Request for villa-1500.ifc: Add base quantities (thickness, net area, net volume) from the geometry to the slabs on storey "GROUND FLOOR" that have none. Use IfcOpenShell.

First a look at what the model holds.

```python
import ifcopenshell
import ifcopenshell.util.element
import ifcopenshell.util.unit

model = ifcopenshell.open("villa-1500.ifc")
print(model.schema)
for unit_type in ("LENGTHUNIT", "AREAUNIT", "VOLUMEUNIT"):
    print(unit_type, ifcopenshell.util.unit.calculate_unit_scale(model, unit_type))
storey = next(s for s in model.by_type("IfcBuildingStorey") if s.Name == "GROUND FLOOR")
slabs = [e for e in ifcopenshell.util.element.get_decomposition(storey) if e.is_a("IfcSlab")]
for e in sorted(slabs, key=lambda e: e.id()):
    print(e.id(), e.is_a(), e.Name, list(ifcopenshell.util.element.get_psets(e, qtos_only=True)), sep=" | ")
```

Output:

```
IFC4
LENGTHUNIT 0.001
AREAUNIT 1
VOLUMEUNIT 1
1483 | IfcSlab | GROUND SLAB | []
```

```python
import ifcopenshell
import ifcopenshell.api.pset
import ifcopenshell.geom
import ifcopenshell.util.element
import ifcopenshell.util.shape
import ifcopenshell.util.unit

model = ifcopenshell.open("villa-1500.ifc")
unit_scale = ifcopenshell.util.unit.calculate_unit_scale(model)
area_scale = ifcopenshell.util.unit.calculate_unit_scale(model, "AREAUNIT")
volume_scale = ifcopenshell.util.unit.calculate_unit_scale(model, "VOLUMEUNIT")
settings = ifcopenshell.geom.settings()

storey = next(s for s in model.by_type("IfcBuildingStorey") if s.Name == "GROUND FLOOR")
slabs = [e for e in ifcopenshell.util.element.get_decomposition(storey) if e.is_a("IfcSlab")]

for e in sorted(slabs, key=lambda e: e.id()):
    if ifcopenshell.util.element.get_psets(e, qtos_only=True, should_inherit=False):
        continue
    # Geometry comes back in metres, in the element's own axes.
    shape = ifcopenshell.geom.create_shape(settings, e)
    values = {
        "Width": ifcopenshell.util.shape.get_z(shape.geometry) / unit_scale,
        "NetArea": ifcopenshell.util.shape.get_footprint_area(shape.geometry) / area_scale,
        "NetVolume": ifcopenshell.util.shape.get_volume(shape.geometry) / volume_scale,
    }
    qto = ifcopenshell.api.pset.add_qto(model, product=e, name="Qto_SlabBaseQuantities")
    ifcopenshell.api.pset.edit_qto(model, qto=qto, properties=values)
    print(e.id(), {k: round(v, 3) for k, v in values.items()})

model.write("villa-1500_v2.ifc")
```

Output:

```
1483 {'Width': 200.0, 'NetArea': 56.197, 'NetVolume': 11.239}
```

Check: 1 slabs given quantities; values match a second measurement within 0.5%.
